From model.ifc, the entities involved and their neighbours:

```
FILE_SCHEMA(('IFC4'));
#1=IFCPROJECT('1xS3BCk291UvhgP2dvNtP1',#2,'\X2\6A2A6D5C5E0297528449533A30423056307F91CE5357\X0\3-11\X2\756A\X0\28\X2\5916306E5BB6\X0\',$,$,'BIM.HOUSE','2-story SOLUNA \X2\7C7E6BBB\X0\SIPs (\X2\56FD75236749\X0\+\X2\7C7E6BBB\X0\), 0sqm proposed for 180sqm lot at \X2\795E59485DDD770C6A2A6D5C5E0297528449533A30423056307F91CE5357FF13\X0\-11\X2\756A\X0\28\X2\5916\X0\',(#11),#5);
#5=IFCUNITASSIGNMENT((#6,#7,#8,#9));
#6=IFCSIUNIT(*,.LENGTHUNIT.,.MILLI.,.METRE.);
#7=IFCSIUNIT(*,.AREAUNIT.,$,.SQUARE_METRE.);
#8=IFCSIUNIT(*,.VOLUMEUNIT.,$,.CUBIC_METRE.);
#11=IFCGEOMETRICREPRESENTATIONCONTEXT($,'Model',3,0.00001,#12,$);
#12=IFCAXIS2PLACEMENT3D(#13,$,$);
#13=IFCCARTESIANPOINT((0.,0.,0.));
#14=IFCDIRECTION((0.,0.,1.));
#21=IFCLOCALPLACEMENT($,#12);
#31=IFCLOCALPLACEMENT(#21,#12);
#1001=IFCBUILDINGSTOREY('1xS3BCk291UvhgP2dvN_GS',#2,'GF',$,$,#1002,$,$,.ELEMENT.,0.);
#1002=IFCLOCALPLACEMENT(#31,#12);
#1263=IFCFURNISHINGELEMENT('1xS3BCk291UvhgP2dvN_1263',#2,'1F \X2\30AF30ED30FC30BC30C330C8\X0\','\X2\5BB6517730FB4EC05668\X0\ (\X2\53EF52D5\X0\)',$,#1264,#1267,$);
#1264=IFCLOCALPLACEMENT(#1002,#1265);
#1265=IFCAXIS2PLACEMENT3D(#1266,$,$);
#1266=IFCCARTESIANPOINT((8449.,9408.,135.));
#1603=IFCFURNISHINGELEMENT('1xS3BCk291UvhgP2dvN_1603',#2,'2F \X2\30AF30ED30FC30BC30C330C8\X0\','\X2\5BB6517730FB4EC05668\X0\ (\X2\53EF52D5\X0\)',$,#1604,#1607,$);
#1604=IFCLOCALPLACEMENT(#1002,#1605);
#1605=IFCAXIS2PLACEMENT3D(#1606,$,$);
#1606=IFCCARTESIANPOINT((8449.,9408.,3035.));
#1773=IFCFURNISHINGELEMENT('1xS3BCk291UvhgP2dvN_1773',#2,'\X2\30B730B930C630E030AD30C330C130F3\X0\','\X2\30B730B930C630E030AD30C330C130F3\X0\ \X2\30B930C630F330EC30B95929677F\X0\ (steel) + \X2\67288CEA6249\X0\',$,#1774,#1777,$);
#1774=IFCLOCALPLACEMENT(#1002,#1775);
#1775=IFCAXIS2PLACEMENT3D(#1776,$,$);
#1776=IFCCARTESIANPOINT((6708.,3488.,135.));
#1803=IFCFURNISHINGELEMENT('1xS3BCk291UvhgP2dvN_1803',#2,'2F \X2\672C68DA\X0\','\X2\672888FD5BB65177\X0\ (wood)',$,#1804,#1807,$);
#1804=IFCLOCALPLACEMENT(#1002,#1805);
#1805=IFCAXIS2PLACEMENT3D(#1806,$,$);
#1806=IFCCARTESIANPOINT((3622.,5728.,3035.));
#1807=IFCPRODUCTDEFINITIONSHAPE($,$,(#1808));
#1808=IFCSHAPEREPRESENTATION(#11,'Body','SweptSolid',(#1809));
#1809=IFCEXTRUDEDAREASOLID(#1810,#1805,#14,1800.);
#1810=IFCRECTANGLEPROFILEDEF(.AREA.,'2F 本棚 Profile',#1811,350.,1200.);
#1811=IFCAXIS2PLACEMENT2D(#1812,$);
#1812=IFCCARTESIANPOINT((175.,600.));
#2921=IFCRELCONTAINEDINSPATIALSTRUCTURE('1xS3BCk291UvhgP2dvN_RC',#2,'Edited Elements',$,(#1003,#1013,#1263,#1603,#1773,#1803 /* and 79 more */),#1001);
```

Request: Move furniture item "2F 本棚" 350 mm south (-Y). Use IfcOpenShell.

```python
import ifcopenshell
import ifcopenshell.api.geometry
import ifcopenshell.util.placement

model = ifcopenshell.open("model.ifc")

item = model.by_id(1803)
matrix = ifcopenshell.util.placement.get_local_placement(item.ObjectPlacement)
matrix[1, 3] -= 350.0
ifcopenshell.api.geometry.edit_object_placement(model, product=item, matrix=matrix, is_si=False)

print(ifcopenshell.util.placement.get_local_placement(item.ObjectPlacement).round(3) + 0.0)

model.write("model_edited.ifc")
```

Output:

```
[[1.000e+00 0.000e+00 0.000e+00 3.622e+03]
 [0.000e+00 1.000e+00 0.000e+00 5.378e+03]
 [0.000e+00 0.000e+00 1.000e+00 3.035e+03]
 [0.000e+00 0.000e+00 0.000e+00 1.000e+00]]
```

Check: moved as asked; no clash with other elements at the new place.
